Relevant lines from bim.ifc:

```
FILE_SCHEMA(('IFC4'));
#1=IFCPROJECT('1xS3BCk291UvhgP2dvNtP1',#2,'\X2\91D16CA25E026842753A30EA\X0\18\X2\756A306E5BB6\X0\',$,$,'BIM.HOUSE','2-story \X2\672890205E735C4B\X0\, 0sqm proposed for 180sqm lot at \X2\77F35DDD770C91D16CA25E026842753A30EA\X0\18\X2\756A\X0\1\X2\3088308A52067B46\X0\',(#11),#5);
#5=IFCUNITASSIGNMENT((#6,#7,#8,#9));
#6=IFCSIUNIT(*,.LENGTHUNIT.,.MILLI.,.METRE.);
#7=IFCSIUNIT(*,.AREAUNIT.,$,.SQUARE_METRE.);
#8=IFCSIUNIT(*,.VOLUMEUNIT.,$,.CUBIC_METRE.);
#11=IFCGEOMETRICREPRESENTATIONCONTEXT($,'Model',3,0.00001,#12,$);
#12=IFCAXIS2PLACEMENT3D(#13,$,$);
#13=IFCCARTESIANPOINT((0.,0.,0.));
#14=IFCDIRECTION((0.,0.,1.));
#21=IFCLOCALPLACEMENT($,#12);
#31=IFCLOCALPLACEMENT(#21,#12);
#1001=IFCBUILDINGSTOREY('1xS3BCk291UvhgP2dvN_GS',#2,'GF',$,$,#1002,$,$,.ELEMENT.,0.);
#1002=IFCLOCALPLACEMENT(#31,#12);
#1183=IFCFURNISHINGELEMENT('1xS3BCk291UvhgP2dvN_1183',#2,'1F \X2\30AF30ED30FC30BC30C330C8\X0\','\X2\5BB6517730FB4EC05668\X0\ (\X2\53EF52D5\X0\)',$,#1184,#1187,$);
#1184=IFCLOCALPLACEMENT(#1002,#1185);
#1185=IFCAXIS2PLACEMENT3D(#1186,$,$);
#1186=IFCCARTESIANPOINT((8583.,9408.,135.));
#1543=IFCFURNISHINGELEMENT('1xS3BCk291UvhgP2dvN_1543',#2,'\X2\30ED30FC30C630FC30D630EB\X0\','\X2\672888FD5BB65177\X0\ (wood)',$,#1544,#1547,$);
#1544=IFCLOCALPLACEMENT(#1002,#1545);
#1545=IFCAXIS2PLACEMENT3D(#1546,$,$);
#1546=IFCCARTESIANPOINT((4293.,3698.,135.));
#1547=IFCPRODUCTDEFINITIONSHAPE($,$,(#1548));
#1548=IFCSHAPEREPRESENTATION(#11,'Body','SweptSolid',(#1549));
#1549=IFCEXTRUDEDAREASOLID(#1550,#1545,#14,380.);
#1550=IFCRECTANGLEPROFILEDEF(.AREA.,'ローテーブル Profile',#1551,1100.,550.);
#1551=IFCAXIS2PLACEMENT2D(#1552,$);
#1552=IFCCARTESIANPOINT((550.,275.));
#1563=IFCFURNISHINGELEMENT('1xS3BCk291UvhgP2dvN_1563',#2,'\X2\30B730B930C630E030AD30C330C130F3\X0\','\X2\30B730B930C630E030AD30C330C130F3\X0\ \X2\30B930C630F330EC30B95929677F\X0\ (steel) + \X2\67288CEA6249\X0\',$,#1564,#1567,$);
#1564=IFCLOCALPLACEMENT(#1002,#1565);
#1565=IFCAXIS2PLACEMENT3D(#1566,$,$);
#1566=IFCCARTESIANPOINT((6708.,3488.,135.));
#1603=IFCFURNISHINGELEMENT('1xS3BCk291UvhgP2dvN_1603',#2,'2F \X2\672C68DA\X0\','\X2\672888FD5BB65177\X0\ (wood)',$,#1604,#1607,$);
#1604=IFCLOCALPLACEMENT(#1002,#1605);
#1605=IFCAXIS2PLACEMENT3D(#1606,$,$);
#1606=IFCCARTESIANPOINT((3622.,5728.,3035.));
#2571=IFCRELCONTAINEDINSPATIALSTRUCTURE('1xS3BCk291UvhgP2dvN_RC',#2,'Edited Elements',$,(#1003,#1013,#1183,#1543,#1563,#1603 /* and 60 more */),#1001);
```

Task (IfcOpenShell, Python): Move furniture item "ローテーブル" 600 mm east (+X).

```python
import ifcopenshell
import ifcopenshell.api.geometry
import ifcopenshell.util.placement

model = ifcopenshell.open("bim.ifc")

item = model.by_id(1543)
matrix = ifcopenshell.util.placement.get_local_placement(item.ObjectPlacement)
matrix[0, 3] += 600.0
ifcopenshell.api.geometry.edit_object_placement(model, product=item, matrix=matrix, is_si=False)

print(ifcopenshell.util.placement.get_local_placement(item.ObjectPlacement).round(3) + 0.0)

model.write("bim-out.ifc")
```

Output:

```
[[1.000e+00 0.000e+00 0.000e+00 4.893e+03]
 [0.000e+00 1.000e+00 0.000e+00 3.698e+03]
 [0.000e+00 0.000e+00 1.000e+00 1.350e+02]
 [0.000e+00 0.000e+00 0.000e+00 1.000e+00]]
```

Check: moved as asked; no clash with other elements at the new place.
